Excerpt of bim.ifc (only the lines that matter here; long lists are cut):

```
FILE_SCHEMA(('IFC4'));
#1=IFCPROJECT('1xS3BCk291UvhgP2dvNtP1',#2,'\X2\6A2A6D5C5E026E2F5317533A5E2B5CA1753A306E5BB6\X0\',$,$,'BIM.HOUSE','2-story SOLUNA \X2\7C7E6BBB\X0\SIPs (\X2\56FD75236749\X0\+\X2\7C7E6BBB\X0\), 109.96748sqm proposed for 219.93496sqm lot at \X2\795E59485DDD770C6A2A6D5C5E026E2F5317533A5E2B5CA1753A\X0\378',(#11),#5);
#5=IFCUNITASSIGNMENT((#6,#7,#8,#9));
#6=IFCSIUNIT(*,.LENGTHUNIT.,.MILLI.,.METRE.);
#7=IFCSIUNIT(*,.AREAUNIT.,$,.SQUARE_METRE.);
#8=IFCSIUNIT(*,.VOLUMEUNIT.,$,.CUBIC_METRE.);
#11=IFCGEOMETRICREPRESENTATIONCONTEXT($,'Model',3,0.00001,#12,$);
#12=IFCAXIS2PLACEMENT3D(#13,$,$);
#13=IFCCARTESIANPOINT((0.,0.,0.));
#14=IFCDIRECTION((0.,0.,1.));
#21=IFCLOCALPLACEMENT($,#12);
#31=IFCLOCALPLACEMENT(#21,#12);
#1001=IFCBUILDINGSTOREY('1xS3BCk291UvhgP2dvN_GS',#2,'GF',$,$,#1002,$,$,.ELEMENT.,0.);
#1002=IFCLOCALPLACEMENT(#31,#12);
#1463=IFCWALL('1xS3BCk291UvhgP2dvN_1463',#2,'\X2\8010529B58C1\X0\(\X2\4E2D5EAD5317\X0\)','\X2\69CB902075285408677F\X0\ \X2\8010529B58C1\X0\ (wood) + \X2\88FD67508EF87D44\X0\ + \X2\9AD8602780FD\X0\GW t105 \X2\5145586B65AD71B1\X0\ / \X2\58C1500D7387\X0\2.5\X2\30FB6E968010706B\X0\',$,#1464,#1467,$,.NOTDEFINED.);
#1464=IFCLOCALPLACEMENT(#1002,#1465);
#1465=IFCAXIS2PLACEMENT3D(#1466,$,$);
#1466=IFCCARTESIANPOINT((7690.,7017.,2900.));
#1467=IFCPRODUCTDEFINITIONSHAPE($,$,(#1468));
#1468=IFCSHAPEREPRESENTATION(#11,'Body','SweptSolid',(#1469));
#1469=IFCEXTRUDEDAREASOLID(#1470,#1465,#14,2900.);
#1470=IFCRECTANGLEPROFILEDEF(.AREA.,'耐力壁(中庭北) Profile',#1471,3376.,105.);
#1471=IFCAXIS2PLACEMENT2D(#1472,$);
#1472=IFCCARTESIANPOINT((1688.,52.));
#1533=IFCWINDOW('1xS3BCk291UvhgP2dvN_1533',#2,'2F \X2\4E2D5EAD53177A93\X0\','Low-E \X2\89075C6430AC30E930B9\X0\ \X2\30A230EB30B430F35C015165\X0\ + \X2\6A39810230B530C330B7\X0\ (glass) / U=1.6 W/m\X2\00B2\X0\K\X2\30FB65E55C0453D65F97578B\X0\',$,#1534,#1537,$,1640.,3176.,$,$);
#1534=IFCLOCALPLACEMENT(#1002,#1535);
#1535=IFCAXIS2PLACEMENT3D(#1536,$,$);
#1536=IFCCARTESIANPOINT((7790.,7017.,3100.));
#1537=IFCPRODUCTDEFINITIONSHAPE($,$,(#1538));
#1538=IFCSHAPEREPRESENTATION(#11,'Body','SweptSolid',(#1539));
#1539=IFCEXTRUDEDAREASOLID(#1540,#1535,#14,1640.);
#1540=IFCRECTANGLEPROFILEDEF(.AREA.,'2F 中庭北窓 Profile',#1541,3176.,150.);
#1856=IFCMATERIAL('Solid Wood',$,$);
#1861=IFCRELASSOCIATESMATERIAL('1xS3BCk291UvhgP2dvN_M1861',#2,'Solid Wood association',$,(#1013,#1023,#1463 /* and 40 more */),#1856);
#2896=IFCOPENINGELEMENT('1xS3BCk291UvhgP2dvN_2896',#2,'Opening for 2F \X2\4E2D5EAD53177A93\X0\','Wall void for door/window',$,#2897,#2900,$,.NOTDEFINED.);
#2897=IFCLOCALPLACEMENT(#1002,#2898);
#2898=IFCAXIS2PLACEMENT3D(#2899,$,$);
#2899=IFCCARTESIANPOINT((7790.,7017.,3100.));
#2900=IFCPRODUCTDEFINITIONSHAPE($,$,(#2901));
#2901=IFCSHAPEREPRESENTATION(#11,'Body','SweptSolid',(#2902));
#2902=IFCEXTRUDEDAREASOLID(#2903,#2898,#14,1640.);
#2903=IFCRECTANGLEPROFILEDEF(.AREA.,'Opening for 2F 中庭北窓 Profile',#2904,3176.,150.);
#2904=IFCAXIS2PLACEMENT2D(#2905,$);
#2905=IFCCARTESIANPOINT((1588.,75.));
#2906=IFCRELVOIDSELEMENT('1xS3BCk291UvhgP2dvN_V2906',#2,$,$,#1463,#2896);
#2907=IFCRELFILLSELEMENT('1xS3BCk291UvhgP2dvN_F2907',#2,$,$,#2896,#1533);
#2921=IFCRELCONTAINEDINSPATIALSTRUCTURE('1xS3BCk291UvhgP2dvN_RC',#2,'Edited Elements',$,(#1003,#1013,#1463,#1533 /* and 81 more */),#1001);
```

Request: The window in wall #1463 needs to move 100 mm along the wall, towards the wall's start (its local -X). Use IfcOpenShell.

```python
import ifcopenshell
import ifcopenshell.api.geometry
import ifcopenshell.util.placement
import ifcopenshell.util.unit

model = ifcopenshell.open("bim.ifc")
unit_scale = ifcopenshell.util.unit.calculate_unit_scale(model)

window = model.by_guid("1xS3BCk291UvhgP2dvN_1533")
opening = window.FillsVoids[0].RelatingOpeningElement
wall = opening.VoidsElements[0].RelatingBuildingElement

wall_matrix = ifcopenshell.util.placement.get_local_placement(wall.ObjectPlacement)
shift = wall_matrix[:3, 0] * -0.1 / unit_scale
before = ifcopenshell.util.placement.get_local_placement(window.ObjectPlacement)[:3, 3].copy()

# The window is not placed relative to its opening, so move both.
for product in (opening, window):
    matrix = ifcopenshell.util.placement.get_local_placement(product.ObjectPlacement)
    matrix[:3, 3] += shift
    ifcopenshell.api.geometry.edit_object_placement(model, product=product, matrix=matrix, is_si=False)

after = ifcopenshell.util.placement.get_local_placement(window.ObjectPlacement)[:3, 3]
print("window moved by", (after - before).round(3) + 0.0)

model.write("bim_v2.ifc")
```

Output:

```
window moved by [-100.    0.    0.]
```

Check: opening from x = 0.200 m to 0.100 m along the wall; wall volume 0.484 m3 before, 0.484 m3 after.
